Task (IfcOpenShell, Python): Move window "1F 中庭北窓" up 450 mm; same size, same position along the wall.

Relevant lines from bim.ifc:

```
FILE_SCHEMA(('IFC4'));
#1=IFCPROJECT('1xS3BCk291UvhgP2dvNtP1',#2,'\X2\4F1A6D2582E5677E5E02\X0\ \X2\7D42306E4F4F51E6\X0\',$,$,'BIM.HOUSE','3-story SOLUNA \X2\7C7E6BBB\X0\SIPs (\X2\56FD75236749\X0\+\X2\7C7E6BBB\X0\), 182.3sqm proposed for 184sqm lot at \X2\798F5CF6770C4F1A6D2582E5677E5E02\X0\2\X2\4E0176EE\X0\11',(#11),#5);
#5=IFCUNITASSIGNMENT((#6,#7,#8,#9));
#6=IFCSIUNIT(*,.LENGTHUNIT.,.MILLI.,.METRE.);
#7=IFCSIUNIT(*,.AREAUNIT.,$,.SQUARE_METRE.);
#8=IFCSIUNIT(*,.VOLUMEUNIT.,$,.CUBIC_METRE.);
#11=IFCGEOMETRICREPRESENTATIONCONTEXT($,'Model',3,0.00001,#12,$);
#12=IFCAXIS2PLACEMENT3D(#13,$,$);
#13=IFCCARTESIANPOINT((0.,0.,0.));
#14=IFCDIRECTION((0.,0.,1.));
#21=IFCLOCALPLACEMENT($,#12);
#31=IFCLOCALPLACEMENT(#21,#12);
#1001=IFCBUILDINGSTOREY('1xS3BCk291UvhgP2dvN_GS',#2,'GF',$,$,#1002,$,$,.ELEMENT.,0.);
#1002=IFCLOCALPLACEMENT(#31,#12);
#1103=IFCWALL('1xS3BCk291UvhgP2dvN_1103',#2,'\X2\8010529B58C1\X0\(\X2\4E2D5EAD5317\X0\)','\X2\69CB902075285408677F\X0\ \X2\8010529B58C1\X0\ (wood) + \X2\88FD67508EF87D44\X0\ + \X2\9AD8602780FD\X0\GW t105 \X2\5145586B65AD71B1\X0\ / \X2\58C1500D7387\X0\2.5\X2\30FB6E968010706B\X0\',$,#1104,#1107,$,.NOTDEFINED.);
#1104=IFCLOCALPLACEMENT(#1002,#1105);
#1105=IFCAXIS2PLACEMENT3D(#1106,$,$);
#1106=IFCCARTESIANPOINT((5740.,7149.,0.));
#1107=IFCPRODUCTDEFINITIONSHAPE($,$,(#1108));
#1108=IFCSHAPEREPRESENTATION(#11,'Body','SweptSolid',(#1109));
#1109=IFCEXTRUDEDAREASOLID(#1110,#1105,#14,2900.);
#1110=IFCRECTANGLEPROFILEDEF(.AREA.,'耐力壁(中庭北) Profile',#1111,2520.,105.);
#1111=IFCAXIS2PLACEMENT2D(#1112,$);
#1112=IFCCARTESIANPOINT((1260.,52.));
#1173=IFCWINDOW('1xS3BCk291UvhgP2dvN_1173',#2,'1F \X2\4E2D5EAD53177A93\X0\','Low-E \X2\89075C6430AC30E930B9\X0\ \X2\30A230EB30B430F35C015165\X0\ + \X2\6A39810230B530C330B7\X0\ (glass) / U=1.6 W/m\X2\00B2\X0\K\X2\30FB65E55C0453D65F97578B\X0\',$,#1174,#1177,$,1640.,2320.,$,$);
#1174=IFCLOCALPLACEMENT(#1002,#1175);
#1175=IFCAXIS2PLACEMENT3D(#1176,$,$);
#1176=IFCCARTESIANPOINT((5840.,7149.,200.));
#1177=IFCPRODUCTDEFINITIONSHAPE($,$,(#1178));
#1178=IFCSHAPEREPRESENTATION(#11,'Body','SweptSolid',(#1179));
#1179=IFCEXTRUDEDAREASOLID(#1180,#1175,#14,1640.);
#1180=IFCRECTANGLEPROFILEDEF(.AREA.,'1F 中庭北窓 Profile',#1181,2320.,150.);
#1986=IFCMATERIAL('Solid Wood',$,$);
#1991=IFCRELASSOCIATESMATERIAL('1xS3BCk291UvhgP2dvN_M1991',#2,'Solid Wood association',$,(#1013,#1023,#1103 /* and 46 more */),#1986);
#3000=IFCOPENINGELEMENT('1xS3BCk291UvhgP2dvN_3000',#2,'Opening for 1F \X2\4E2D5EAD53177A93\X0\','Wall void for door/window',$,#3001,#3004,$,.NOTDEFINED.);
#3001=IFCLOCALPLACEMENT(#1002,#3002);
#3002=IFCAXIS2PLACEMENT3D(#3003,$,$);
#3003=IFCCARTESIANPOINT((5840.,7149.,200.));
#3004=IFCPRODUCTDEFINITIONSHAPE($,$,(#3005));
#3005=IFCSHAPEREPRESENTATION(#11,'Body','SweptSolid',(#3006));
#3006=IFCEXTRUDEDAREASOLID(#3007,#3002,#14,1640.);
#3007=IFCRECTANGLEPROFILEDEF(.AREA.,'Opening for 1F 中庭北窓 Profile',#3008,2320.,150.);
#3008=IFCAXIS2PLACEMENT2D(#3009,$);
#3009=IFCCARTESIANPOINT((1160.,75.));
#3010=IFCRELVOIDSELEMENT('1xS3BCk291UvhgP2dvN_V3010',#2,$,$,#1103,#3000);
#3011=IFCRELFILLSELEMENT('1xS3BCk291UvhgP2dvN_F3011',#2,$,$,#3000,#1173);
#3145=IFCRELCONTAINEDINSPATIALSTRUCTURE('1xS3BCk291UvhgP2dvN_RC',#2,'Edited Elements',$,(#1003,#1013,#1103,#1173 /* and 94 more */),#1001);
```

```python
import numpy as np
import ifcopenshell
import ifcopenshell.api.geometry
import ifcopenshell.util.placement
import ifcopenshell.util.unit

model = ifcopenshell.open("bim.ifc")
unit_scale = ifcopenshell.util.unit.calculate_unit_scale(model)

window = model.by_guid("1xS3BCk291UvhgP2dvN_1173")
opening = window.FillsVoids[0].RelatingOpeningElement
dz = 450.0

shift = np.array([0.0, 0.0, dz])
# The window is not placed relative to its opening, so move both.
for product in (opening, window):
    matrix = ifcopenshell.util.placement.get_local_placement(product.ObjectPlacement)
    matrix[:3, 3] += shift
    ifcopenshell.api.geometry.edit_object_placement(model, product=product, matrix=matrix, is_si=False)

print(f"moved by {dz * unit_scale:+.3f} m")

model.write("bim_rev.ifc")
```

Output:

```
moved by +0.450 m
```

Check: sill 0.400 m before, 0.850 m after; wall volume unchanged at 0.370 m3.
